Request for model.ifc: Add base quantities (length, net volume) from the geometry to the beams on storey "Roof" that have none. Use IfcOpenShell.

First a look at what the model holds.

```python
import ifcopenshell
import ifcopenshell.util.element
import ifcopenshell.util.unit

model = ifcopenshell.open("model.ifc")
print(model.schema)
for unit_type in ("LENGTHUNIT", "AREAUNIT", "VOLUMEUNIT"):
    print(unit_type, ifcopenshell.util.unit.calculate_unit_scale(model, unit_type))
storey = next(s for s in model.by_type("IfcBuildingStorey") if s.Name == "Roof")
beams = [e for e in ifcopenshell.util.element.get_decomposition(storey) if e.is_a("IfcBeam")]
for e in sorted(beams, key=lambda e: e.id()):
    print(e.id(), e.is_a(), e.Name, list(ifcopenshell.util.element.get_psets(e, qtos_only=True)), sep=" | ")
```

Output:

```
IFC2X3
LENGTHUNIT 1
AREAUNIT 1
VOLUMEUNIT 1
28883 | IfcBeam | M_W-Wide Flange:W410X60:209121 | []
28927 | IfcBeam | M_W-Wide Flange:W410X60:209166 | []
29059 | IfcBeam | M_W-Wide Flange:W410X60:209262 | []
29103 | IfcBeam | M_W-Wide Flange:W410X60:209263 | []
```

```python
import ifcopenshell
import ifcopenshell.api.pset
import ifcopenshell.geom
import ifcopenshell.util.element
import ifcopenshell.util.shape
import ifcopenshell.util.unit

model = ifcopenshell.open("model.ifc")
unit_scale = ifcopenshell.util.unit.calculate_unit_scale(model)
volume_scale = ifcopenshell.util.unit.calculate_unit_scale(model, "VOLUMEUNIT")
settings = ifcopenshell.geom.settings()

storey = next(s for s in model.by_type("IfcBuildingStorey") if s.Name == "Roof")
beams = [e for e in ifcopenshell.util.element.get_decomposition(storey) if e.is_a("IfcBeam")]

for e in sorted(beams, key=lambda e: e.id()):
    if ifcopenshell.util.element.get_psets(e, qtos_only=True, should_inherit=False):
        continue
    # Geometry comes back in metres, in the element's own axes.
    shape = ifcopenshell.geom.create_shape(settings, e)
    values = {
        "Length": ifcopenshell.util.shape.get_max_xyz(shape.geometry) / unit_scale,
        "NetVolume": ifcopenshell.util.shape.get_volume(shape.geometry) / volume_scale,
    }
    qto = ifcopenshell.api.pset.add_qto(model, product=e, name="BaseQuantities")
    ifcopenshell.api.pset.edit_qto(model, qto=qto, properties=values)
    print(e.id(), {k: round(v, 3) for k, v in values.items()})

model.write("model_rev.ifc")
```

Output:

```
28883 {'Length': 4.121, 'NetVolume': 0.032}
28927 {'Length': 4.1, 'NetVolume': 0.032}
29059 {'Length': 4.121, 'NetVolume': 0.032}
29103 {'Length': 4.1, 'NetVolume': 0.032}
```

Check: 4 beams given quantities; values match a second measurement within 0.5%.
